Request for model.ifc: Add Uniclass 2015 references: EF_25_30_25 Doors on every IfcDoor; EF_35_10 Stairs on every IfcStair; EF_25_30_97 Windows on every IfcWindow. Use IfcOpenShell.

First a look at what the model holds.

```python
import ifcopenshell

model = ifcopenshell.open("model.ifc")
print(model.schema)
print("classifications:", [c.Name for c in model.by_type("IfcClassification")])
for ifc_class in ("IfcDoor", "IfcRoof", "IfcStair", "IfcWall", "IfcWindow"):
    print(ifc_class, len(model.by_type(ifc_class)))
```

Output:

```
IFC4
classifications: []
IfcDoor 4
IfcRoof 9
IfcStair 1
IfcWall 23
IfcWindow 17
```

```python
import ifcopenshell
import ifcopenshell.api.classification

model = ifcopenshell.open("model.ifc")

system = ifcopenshell.api.classification.add_classification(model, classification="Uniclass 2015")

codes = {
    "IfcDoor": ("EF_25_30_25", "Doors"),
    "IfcStair": ("EF_35_10", "Stairs"),
    "IfcWindow": ("EF_25_30_97", "Windows"),
}
for ifc_class, (code, name) in codes.items():
    products = model.by_type(ifc_class)
    ifcopenshell.api.classification.add_reference(
        model, products=products, classification=system, identification=code, name=name
    )
    print(code, len(products))

model.write("model_updated.ifc")
```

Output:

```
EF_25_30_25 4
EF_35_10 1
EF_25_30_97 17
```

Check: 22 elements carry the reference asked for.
